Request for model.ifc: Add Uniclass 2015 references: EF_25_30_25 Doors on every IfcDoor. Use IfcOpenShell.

First a look at what the model holds.

```python
import ifcopenshell

model = ifcopenshell.open("model.ifc")
print(model.schema)
print("classifications:", [c.Name for c in model.by_type("IfcClassification")])
for ifc_class in ("IfcDoor", "IfcRoof", "IfcStair", "IfcWall", "IfcWindow"):
    print(ifc_class, len(model.by_type(ifc_class)))
```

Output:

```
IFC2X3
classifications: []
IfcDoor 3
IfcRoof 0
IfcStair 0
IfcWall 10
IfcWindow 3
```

```python
import ifcopenshell
import ifcopenshell.api.classification

model = ifcopenshell.open("model.ifc")

# IFC2X3 requires Source and Edition and has no link from the project to the system.
system = model.create_entity("IfcClassification", Source="NBS", Edition="2015", Name="Uniclass 2015")

codes = {
    "IfcDoor": ("EF_25_30_25", "Doors"),
}
for ifc_class, (code, name) in codes.items():
    products = model.by_type(ifc_class)
    ifcopenshell.api.classification.add_reference(
        model, products=products, classification=system, identification=code, name=name
    )
    print(code, len(products))

model.write("model_edited.ifc")
```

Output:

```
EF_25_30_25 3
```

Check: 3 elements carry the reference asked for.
